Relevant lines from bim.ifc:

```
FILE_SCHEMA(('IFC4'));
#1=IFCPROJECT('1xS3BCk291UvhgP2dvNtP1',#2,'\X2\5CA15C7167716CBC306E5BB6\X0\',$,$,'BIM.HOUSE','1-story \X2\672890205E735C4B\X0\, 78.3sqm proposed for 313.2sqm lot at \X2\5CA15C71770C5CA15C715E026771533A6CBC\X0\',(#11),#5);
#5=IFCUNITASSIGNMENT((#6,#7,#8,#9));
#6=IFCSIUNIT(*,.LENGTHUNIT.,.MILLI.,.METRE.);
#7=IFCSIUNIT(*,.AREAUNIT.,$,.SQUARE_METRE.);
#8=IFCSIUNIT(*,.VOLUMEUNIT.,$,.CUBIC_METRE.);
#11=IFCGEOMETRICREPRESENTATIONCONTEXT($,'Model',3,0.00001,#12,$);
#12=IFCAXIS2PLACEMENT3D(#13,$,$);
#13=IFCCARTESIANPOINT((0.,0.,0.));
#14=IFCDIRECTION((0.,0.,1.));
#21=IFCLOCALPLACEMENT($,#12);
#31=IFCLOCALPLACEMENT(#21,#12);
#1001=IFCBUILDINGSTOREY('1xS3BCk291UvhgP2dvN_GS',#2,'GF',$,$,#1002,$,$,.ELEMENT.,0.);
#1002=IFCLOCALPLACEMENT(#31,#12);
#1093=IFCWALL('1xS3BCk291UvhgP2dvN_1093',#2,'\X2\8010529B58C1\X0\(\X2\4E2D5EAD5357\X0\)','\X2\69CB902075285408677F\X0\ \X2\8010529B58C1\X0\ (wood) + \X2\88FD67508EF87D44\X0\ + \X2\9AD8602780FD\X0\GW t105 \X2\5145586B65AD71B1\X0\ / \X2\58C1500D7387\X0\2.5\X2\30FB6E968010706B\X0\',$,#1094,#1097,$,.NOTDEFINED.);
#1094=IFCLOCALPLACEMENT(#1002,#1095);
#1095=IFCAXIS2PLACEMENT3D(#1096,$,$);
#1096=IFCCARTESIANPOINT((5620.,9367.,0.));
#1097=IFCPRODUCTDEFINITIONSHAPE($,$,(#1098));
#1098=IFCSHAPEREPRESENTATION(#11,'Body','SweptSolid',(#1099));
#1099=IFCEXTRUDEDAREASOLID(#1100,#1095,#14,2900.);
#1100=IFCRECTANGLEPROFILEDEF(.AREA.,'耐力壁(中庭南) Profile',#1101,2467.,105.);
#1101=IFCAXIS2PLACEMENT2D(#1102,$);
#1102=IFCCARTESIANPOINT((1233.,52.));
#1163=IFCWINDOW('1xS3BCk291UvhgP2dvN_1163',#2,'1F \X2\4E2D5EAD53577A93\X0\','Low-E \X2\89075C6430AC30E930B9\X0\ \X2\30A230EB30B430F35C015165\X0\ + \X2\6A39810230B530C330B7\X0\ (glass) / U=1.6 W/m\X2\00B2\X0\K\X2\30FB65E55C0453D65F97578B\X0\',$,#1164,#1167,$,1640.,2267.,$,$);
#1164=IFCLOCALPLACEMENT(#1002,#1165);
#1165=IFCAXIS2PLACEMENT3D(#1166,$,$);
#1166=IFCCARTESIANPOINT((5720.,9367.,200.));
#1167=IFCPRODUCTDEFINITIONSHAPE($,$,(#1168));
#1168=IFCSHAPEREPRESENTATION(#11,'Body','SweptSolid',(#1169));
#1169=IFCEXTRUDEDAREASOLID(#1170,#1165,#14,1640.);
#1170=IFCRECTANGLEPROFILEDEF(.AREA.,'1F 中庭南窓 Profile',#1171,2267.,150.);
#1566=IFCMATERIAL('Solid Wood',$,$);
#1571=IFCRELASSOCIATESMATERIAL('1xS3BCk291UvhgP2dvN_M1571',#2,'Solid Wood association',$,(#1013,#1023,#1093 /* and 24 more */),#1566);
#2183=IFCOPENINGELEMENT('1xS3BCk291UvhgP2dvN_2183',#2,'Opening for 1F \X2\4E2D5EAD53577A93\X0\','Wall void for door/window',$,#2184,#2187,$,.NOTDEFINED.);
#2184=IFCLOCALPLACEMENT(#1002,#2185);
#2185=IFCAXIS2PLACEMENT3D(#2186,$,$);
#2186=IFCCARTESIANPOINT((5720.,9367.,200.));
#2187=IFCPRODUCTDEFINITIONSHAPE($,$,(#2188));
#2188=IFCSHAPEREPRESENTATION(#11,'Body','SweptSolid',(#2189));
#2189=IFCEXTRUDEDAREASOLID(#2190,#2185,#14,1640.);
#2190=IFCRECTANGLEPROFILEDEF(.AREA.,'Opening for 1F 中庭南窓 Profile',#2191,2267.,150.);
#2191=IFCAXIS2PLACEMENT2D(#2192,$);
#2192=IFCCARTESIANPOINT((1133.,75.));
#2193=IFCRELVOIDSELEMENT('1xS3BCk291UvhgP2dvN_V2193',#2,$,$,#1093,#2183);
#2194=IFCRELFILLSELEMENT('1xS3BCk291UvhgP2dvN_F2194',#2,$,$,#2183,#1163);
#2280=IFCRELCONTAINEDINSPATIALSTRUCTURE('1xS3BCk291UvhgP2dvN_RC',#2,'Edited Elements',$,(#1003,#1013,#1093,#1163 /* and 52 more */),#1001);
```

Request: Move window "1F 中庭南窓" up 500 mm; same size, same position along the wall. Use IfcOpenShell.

```python
import numpy as np
import ifcopenshell
import ifcopenshell.api.geometry
import ifcopenshell.util.placement
import ifcopenshell.util.unit

model = ifcopenshell.open("bim.ifc")
unit_scale = ifcopenshell.util.unit.calculate_unit_scale(model)

window = model.by_id(1163)
opening = window.FillsVoids[0].RelatingOpeningElement
dz = 500.0

shift = np.array([0.0, 0.0, dz])
# The window is not placed relative to its opening, so move both.
for product in (opening, window):
    matrix = ifcopenshell.util.placement.get_local_placement(product.ObjectPlacement)
    matrix[:3, 3] += shift
    ifcopenshell.api.geometry.edit_object_placement(model, product=product, matrix=matrix, is_si=False)

print(f"moved by {dz * unit_scale:+.3f} m")

model.write("bim_updated.ifc")
```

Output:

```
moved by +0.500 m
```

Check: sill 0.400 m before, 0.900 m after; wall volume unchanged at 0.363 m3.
